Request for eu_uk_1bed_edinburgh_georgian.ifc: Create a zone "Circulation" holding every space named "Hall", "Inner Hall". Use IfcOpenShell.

First a look at what the model holds.

```python
import ifcopenshell

model = ifcopenshell.open("eu_uk_1bed_edinburgh_georgian.ifc")
print(model.schema)
seen = {}
for space in model.by_type("IfcSpace"):
    seen[space.LongName] = seen.get(space.LongName, 0) + 1
for name, count in sorted(seen.items(), key=str):
    print(count, "x", name)
print("zones:", [z.Name for z in model.by_type("IfcZone")][:20])
```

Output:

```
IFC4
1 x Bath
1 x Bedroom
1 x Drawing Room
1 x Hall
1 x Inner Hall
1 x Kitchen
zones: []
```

```python
import ifcopenshell
import ifcopenshell.api.group
import ifcopenshell.api.root

model = ifcopenshell.open("eu_uk_1bed_edinburgh_georgian.ifc")

names = {"Hall", "Inner Hall"}
spaces = [s for s in model.by_type("IfcSpace") if s.LongName in names]

zone = ifcopenshell.api.root.create_entity(model, ifc_class="IfcZone", name="Circulation")
ifcopenshell.api.group.assign_group(model, products=spaces, group=zone)
print(len(spaces), "spaces in", zone.Name)

model.write("eu_uk_1bed_edinburgh_georgian_edited.ifc")
```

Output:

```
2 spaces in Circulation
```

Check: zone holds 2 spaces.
